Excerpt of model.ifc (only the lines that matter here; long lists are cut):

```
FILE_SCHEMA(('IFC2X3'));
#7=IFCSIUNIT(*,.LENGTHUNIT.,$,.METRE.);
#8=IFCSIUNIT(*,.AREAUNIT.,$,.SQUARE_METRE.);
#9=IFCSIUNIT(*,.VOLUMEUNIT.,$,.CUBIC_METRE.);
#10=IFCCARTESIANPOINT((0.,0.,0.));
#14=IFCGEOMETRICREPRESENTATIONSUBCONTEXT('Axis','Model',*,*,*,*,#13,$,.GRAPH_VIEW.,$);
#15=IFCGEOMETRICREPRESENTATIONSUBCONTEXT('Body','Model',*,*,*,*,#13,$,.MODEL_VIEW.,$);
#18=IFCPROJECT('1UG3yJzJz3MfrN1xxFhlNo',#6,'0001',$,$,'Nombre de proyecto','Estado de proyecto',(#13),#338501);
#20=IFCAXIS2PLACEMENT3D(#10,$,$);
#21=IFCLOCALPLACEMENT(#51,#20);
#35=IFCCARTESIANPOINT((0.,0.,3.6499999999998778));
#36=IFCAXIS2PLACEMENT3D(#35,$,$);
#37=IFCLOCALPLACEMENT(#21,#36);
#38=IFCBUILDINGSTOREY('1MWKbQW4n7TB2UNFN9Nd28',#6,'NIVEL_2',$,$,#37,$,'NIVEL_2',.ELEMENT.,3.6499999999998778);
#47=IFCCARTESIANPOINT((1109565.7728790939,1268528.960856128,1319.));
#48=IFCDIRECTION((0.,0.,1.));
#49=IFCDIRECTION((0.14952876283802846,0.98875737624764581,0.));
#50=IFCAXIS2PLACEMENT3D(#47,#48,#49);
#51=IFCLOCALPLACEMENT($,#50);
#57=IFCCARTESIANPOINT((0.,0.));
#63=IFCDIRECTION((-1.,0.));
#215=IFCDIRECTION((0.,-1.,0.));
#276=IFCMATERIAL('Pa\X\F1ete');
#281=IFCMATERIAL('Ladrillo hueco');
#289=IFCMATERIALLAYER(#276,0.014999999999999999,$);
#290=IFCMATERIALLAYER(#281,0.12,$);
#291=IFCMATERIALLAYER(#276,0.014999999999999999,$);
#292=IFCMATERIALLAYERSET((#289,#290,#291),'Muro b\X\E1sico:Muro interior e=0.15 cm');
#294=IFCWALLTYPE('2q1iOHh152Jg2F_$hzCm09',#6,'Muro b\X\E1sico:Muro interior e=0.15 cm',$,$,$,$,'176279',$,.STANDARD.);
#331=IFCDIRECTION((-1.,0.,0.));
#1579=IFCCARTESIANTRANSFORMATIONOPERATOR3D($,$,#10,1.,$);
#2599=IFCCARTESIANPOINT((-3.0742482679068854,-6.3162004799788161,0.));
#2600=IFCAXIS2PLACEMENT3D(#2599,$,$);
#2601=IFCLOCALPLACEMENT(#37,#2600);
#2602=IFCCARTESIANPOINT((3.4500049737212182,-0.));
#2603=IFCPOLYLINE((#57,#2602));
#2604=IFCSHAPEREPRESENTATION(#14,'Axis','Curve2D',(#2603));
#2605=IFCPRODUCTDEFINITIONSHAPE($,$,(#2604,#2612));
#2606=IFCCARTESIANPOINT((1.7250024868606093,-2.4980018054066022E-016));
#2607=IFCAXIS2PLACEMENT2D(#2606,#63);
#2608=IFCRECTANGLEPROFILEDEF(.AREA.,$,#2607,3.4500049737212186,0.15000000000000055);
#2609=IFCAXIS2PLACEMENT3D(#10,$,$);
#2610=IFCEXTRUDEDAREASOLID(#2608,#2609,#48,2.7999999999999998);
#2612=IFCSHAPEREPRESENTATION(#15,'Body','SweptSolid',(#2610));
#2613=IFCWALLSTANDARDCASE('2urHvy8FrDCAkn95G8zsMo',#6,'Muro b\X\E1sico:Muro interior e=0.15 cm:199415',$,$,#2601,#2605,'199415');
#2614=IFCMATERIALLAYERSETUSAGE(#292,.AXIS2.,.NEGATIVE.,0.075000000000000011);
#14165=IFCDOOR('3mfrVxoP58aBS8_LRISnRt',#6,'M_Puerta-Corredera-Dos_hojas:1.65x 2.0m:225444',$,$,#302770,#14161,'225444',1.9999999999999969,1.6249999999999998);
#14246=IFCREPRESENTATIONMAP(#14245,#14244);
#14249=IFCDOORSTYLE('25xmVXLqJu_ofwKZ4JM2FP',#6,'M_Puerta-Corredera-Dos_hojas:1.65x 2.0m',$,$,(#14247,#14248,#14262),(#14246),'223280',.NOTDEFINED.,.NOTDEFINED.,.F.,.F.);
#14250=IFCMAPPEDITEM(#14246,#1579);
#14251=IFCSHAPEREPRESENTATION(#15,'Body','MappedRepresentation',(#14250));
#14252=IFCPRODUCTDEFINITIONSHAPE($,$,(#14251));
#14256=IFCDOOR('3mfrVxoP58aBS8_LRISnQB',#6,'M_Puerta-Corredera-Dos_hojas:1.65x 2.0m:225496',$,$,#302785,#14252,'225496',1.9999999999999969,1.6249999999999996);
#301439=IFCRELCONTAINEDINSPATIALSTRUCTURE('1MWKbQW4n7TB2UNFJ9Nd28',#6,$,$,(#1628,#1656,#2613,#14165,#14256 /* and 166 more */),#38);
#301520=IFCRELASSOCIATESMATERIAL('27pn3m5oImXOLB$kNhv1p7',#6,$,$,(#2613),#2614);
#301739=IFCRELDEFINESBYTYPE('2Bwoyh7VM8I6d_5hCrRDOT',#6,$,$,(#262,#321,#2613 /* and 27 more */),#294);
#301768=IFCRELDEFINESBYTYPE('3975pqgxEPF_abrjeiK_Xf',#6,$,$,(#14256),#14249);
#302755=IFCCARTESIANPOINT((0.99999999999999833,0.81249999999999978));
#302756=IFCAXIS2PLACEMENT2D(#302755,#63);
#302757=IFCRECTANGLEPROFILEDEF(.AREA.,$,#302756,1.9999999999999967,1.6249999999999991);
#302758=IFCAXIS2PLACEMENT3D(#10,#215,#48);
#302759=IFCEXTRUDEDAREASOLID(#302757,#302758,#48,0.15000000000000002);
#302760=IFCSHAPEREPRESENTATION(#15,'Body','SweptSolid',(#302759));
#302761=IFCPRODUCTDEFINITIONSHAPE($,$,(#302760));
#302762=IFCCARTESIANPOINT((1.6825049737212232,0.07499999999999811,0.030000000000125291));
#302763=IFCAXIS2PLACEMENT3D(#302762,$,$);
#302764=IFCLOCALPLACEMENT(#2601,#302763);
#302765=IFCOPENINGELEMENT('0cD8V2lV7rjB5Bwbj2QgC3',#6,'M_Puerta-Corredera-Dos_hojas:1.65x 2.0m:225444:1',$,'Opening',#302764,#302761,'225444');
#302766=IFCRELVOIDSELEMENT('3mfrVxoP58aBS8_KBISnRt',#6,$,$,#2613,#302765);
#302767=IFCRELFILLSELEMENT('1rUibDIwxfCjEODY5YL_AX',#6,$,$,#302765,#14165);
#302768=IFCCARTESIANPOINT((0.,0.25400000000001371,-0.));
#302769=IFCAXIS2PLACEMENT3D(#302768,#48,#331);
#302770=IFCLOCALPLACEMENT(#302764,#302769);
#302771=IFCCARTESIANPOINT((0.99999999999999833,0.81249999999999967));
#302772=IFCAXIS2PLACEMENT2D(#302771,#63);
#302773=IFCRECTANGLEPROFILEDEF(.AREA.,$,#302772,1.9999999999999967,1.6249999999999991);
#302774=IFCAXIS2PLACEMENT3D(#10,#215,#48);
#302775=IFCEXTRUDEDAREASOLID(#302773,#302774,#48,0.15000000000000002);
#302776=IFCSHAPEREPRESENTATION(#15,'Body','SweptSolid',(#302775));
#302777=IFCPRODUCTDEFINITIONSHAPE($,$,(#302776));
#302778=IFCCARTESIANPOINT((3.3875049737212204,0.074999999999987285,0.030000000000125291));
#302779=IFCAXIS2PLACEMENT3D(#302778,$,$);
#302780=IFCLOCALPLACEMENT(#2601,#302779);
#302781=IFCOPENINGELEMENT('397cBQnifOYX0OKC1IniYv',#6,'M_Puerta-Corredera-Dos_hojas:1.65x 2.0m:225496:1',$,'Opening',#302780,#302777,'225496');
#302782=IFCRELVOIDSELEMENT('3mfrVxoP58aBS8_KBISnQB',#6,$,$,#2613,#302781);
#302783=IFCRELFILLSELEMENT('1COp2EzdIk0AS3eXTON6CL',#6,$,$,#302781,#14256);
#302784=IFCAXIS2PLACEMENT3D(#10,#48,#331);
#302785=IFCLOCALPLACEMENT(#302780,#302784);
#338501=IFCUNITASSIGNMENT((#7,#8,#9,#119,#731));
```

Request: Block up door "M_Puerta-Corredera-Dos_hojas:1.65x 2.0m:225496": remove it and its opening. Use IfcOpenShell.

```python
import ifcopenshell
import ifcopenshell.api.feature
import ifcopenshell.api.root
import ifcopenshell.geom
import ifcopenshell.util.shape

model = ifcopenshell.open("model.ifc")
settings = ifcopenshell.geom.settings()


def volume(element):
    """Net volume in cubic metres, openings subtracted."""
    shape = ifcopenshell.geom.create_shape(settings, element)
    return ifcopenshell.util.shape.get_volume(shape.geometry)


door = model.by_guid("3mfrVxoP58aBS8_LRISnQB")
opening = door.FillsVoids[0].RelatingOpeningElement
wall = opening.VoidsElements[0].RelatingBuildingElement
before = volume(wall)

ifcopenshell.api.root.remove_product(model, product=door)
ifcopenshell.api.feature.remove_feature(model, feature=opening)

after = volume(wall)

print(f"wall volume {before:.3f} -> {after:.3f} m3")

model.write("model_updated.ifc")
```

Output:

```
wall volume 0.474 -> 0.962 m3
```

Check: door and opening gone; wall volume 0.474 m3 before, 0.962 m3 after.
